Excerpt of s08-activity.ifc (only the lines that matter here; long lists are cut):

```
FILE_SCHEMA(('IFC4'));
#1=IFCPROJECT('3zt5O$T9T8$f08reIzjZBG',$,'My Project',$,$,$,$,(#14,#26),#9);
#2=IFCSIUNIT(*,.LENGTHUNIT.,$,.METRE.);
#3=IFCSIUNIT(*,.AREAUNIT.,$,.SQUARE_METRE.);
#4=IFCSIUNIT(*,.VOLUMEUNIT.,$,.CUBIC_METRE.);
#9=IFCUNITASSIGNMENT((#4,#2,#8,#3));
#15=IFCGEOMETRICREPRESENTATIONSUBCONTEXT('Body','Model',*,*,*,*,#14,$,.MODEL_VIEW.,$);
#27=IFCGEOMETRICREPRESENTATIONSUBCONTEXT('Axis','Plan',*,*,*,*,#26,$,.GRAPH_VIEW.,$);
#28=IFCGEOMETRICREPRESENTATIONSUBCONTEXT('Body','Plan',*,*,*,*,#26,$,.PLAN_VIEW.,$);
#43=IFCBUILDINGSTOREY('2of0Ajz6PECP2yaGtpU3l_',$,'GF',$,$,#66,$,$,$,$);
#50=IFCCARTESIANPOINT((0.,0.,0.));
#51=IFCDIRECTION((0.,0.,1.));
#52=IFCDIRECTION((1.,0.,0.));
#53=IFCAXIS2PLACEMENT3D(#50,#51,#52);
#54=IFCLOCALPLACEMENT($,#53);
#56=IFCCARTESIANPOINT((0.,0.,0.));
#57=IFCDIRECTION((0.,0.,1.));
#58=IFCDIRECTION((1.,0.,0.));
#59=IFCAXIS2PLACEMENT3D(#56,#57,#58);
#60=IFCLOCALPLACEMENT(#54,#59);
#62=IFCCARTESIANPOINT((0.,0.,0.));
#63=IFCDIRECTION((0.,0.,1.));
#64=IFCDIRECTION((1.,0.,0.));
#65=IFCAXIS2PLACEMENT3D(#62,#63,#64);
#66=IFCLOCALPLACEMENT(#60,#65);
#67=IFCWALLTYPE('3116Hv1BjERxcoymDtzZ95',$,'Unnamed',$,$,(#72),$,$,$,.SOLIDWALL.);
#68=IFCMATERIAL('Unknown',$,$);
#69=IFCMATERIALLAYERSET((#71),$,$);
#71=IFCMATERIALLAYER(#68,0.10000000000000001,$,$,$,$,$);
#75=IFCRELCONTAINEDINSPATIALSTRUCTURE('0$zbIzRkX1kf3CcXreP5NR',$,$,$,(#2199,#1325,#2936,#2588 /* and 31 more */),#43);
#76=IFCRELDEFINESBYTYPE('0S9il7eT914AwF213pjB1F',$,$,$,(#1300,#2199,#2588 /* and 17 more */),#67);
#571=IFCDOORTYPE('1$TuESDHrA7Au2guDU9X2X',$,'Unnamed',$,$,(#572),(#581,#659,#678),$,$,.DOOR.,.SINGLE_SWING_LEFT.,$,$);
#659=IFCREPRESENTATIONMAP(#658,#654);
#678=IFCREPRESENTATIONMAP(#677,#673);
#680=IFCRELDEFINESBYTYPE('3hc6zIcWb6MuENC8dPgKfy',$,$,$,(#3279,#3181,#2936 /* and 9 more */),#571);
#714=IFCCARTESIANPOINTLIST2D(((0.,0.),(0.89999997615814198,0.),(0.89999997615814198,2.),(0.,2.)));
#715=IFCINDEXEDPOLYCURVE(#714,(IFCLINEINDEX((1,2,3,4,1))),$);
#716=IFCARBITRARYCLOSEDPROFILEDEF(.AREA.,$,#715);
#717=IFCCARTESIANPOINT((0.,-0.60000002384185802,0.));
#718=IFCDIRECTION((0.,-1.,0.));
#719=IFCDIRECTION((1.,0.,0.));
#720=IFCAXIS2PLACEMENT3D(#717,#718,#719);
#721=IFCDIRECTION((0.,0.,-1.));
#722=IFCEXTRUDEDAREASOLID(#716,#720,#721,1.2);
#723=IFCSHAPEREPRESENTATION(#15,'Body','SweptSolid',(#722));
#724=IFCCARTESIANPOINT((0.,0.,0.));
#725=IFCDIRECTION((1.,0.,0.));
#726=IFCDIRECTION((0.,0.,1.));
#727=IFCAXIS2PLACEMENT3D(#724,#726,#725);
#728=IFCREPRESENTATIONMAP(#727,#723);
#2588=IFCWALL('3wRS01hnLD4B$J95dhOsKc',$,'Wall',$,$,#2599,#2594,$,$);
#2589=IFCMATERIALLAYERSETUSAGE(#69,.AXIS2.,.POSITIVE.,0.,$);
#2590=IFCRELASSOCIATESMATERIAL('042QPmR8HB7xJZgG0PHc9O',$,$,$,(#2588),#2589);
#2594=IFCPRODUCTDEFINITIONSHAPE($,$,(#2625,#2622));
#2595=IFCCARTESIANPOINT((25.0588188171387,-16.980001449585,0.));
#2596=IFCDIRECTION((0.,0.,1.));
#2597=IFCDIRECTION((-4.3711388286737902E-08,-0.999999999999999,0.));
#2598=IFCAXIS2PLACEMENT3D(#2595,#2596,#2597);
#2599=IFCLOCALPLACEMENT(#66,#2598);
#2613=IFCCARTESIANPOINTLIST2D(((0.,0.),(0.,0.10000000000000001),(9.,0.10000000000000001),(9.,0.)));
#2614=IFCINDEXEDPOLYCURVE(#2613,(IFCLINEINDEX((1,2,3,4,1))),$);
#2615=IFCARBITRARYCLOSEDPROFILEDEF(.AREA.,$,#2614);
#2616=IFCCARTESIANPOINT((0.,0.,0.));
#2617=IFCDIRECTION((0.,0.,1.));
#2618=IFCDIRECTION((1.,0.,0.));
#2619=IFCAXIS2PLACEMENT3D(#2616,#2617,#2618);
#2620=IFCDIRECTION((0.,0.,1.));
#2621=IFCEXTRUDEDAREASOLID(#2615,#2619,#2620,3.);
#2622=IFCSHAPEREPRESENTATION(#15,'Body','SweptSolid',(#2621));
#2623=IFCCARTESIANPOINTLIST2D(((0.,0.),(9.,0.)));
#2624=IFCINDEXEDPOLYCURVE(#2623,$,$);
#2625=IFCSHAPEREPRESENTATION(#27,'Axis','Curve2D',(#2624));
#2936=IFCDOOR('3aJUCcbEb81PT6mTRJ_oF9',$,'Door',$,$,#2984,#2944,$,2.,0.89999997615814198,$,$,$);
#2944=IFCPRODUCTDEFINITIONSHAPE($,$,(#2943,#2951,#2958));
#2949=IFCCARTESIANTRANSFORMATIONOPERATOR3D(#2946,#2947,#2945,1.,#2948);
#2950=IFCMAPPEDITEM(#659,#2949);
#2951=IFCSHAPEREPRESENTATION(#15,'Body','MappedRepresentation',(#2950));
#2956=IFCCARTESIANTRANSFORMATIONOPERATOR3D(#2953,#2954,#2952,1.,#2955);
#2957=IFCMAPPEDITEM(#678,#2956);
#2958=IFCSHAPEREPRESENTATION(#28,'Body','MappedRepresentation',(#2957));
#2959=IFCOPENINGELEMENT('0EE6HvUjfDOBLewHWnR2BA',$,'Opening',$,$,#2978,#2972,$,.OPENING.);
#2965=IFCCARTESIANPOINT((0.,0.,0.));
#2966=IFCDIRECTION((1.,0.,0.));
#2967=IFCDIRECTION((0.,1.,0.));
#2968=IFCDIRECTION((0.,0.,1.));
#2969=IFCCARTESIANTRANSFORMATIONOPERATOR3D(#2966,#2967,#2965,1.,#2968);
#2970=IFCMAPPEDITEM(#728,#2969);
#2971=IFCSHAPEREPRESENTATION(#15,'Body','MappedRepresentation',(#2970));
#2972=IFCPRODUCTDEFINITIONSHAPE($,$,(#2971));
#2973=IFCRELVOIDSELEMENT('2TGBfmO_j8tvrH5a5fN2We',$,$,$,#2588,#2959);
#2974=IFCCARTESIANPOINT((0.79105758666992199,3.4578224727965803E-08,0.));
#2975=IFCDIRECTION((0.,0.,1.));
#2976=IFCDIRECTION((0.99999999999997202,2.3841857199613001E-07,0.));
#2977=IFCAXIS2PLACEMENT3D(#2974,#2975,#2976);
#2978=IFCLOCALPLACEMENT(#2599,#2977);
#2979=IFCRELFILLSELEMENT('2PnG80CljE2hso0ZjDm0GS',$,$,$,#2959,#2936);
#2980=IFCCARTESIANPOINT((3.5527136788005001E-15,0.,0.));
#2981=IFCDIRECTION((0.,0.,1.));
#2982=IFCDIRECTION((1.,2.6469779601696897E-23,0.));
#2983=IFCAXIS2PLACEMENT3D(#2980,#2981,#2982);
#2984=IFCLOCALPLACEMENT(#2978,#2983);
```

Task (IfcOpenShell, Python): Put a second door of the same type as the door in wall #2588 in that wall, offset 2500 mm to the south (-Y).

```python
import ifcopenshell
import ifcopenshell.api.feature
import ifcopenshell.api.geometry
import ifcopenshell.api.root
import ifcopenshell.geom
import ifcopenshell.util.element
import ifcopenshell.util.placement
import ifcopenshell.util.shape
import ifcopenshell.util.unit

model = ifcopenshell.open("s08-activity.ifc")
unit_scale = ifcopenshell.util.unit.calculate_unit_scale(model)
settings = ifcopenshell.geom.settings()


def volume(element):
    """Net volume in cubic metres, openings subtracted."""
    shape = ifcopenshell.geom.create_shape(settings, element)
    return ifcopenshell.util.shape.get_volume(shape.geometry)


door = model.by_guid("3aJUCcbEb81PT6mTRJ_oF9")
opening = door.FillsVoids[0].RelatingOpeningElement
wall = opening.VoidsElements[0].RelatingBuildingElement
before = volume(wall)
shift = ifcopenshell.util.placement.get_local_placement(wall.ObjectPlacement)[:3, 0] * 2.5 / unit_scale

# copy_class copies the void relationship, type, container and properties, but no geometry.
new_opening = ifcopenshell.api.root.copy_class(model, product=opening)
new_opening.Representation = ifcopenshell.util.element.copy_deep(
    model, opening.Representation, exclude=["IfcGeometricRepresentationContext", "IfcRepresentationMap"]
)
new_door = ifcopenshell.api.root.copy_class(model, product=door)
new_door.Representation = ifcopenshell.util.element.copy_deep(
    model, door.Representation, exclude=["IfcGeometricRepresentationContext", "IfcRepresentationMap"]
)
ifcopenshell.api.feature.add_filling(model, opening=new_opening, element=new_door)

for old, new in ((opening, new_opening), (door, new_door)):
    matrix = ifcopenshell.util.placement.get_local_placement(old.ObjectPlacement)
    matrix[:3, 3] += shift
    ifcopenshell.api.geometry.edit_object_placement(model, product=new, matrix=matrix, is_si=False)

after = volume(wall)

print(f"wall volume {before:.3f} -> {after:.3f} m3")

model.write("s08-activity_updated.ifc")
```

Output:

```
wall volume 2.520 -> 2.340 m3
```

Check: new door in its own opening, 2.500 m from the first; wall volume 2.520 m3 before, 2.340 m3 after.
